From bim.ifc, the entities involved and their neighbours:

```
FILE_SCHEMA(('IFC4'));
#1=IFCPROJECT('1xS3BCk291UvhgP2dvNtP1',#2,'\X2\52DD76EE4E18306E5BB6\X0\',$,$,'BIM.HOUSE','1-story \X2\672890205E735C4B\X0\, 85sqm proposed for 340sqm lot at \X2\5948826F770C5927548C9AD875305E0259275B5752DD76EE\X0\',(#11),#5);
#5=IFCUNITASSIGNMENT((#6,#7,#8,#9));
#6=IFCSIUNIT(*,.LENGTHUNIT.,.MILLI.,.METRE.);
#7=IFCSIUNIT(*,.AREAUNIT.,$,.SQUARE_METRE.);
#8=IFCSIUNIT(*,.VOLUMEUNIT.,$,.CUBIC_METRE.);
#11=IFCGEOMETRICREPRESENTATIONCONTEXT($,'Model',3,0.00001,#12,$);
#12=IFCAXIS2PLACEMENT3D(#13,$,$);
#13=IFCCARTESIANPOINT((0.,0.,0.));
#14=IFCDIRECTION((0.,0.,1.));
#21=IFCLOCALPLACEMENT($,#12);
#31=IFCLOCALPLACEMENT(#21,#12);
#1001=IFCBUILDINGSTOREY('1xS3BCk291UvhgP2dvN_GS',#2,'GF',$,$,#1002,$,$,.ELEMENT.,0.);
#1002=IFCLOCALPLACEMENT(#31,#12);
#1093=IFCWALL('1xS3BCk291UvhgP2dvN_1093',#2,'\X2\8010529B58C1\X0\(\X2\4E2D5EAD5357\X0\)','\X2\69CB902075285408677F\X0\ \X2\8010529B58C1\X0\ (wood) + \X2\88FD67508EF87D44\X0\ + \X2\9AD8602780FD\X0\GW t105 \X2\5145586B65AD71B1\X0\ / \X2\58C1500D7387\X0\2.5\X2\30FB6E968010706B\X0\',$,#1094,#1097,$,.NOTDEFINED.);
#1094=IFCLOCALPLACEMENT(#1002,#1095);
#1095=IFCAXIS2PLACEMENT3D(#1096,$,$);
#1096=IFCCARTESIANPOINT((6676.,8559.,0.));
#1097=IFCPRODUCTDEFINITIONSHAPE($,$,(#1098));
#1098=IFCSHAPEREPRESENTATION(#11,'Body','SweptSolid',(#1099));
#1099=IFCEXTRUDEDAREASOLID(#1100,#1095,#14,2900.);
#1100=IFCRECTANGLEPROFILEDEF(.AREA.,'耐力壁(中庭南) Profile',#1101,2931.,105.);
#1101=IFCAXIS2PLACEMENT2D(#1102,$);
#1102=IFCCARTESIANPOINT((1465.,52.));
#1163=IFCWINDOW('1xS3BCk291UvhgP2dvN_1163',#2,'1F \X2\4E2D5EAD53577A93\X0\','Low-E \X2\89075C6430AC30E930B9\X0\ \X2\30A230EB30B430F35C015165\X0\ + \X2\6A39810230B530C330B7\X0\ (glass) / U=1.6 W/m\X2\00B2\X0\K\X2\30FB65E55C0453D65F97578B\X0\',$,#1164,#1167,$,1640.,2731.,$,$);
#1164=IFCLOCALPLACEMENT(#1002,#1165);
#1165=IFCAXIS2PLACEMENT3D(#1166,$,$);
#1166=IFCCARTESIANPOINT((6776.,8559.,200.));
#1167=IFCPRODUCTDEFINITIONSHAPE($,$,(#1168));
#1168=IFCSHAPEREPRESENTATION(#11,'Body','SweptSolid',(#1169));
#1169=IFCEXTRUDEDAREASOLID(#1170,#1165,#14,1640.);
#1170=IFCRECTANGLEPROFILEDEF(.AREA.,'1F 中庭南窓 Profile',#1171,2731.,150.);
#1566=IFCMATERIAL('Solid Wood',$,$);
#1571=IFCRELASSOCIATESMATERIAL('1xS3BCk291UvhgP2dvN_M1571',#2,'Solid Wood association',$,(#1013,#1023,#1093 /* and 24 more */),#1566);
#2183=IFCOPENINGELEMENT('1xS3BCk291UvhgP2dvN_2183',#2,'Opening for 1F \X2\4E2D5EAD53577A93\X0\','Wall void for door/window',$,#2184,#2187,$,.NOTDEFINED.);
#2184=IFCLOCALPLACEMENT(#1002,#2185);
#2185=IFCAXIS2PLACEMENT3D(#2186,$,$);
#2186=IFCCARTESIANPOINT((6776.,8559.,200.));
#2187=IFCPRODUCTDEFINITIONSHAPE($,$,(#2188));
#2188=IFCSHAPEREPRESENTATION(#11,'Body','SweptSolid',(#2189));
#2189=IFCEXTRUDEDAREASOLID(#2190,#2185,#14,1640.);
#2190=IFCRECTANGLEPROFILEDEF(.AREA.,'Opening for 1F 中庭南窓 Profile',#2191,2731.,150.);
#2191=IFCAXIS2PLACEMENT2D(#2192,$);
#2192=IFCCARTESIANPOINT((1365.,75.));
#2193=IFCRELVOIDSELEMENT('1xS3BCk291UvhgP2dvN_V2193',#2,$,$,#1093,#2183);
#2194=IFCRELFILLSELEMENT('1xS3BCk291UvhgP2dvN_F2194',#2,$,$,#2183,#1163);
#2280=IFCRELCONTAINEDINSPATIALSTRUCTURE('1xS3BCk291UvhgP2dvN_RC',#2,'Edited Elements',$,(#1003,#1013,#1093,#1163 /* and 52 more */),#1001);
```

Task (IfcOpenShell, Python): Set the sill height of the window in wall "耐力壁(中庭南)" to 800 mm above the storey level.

```python
import numpy as np
import ifcopenshell
import ifcopenshell.api.geometry
import ifcopenshell.geom
import ifcopenshell.util.element
import ifcopenshell.util.placement
import ifcopenshell.util.shape
import ifcopenshell.util.unit

model = ifcopenshell.open("bim.ifc")
unit_scale = ifcopenshell.util.unit.calculate_unit_scale(model)

window = model.by_guid("1xS3BCk291UvhgP2dvN_1163")
opening = window.FillsVoids[0].RelatingOpeningElement
storey = ifcopenshell.util.element.get_container(window, ifc_class="IfcBuildingStorey")
level = ifcopenshell.util.placement.get_local_placement(storey.ObjectPlacement)[2, 3]

# The opening's origin need not be at the sill, so measure its lowest point.
shape = ifcopenshell.geom.create_shape(ifcopenshell.geom.settings(), opening)
bottom = ifcopenshell.util.shape.get_shape_bottom_elevation(shape, shape.geometry) / unit_scale
dz = level + 0.8 / unit_scale - bottom

shift = np.array([0.0, 0.0, dz])
# The window is not placed relative to its opening, so move both.
for product in (opening, window):
    matrix = ifcopenshell.util.placement.get_local_placement(product.ObjectPlacement)
    matrix[:3, 3] += shift
    ifcopenshell.api.geometry.edit_object_placement(model, product=product, matrix=matrix, is_si=False)

print(f"moved by {dz * unit_scale:+.3f} m")

model.write("bim_edited.ifc")
```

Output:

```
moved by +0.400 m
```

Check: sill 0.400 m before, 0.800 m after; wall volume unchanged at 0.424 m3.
